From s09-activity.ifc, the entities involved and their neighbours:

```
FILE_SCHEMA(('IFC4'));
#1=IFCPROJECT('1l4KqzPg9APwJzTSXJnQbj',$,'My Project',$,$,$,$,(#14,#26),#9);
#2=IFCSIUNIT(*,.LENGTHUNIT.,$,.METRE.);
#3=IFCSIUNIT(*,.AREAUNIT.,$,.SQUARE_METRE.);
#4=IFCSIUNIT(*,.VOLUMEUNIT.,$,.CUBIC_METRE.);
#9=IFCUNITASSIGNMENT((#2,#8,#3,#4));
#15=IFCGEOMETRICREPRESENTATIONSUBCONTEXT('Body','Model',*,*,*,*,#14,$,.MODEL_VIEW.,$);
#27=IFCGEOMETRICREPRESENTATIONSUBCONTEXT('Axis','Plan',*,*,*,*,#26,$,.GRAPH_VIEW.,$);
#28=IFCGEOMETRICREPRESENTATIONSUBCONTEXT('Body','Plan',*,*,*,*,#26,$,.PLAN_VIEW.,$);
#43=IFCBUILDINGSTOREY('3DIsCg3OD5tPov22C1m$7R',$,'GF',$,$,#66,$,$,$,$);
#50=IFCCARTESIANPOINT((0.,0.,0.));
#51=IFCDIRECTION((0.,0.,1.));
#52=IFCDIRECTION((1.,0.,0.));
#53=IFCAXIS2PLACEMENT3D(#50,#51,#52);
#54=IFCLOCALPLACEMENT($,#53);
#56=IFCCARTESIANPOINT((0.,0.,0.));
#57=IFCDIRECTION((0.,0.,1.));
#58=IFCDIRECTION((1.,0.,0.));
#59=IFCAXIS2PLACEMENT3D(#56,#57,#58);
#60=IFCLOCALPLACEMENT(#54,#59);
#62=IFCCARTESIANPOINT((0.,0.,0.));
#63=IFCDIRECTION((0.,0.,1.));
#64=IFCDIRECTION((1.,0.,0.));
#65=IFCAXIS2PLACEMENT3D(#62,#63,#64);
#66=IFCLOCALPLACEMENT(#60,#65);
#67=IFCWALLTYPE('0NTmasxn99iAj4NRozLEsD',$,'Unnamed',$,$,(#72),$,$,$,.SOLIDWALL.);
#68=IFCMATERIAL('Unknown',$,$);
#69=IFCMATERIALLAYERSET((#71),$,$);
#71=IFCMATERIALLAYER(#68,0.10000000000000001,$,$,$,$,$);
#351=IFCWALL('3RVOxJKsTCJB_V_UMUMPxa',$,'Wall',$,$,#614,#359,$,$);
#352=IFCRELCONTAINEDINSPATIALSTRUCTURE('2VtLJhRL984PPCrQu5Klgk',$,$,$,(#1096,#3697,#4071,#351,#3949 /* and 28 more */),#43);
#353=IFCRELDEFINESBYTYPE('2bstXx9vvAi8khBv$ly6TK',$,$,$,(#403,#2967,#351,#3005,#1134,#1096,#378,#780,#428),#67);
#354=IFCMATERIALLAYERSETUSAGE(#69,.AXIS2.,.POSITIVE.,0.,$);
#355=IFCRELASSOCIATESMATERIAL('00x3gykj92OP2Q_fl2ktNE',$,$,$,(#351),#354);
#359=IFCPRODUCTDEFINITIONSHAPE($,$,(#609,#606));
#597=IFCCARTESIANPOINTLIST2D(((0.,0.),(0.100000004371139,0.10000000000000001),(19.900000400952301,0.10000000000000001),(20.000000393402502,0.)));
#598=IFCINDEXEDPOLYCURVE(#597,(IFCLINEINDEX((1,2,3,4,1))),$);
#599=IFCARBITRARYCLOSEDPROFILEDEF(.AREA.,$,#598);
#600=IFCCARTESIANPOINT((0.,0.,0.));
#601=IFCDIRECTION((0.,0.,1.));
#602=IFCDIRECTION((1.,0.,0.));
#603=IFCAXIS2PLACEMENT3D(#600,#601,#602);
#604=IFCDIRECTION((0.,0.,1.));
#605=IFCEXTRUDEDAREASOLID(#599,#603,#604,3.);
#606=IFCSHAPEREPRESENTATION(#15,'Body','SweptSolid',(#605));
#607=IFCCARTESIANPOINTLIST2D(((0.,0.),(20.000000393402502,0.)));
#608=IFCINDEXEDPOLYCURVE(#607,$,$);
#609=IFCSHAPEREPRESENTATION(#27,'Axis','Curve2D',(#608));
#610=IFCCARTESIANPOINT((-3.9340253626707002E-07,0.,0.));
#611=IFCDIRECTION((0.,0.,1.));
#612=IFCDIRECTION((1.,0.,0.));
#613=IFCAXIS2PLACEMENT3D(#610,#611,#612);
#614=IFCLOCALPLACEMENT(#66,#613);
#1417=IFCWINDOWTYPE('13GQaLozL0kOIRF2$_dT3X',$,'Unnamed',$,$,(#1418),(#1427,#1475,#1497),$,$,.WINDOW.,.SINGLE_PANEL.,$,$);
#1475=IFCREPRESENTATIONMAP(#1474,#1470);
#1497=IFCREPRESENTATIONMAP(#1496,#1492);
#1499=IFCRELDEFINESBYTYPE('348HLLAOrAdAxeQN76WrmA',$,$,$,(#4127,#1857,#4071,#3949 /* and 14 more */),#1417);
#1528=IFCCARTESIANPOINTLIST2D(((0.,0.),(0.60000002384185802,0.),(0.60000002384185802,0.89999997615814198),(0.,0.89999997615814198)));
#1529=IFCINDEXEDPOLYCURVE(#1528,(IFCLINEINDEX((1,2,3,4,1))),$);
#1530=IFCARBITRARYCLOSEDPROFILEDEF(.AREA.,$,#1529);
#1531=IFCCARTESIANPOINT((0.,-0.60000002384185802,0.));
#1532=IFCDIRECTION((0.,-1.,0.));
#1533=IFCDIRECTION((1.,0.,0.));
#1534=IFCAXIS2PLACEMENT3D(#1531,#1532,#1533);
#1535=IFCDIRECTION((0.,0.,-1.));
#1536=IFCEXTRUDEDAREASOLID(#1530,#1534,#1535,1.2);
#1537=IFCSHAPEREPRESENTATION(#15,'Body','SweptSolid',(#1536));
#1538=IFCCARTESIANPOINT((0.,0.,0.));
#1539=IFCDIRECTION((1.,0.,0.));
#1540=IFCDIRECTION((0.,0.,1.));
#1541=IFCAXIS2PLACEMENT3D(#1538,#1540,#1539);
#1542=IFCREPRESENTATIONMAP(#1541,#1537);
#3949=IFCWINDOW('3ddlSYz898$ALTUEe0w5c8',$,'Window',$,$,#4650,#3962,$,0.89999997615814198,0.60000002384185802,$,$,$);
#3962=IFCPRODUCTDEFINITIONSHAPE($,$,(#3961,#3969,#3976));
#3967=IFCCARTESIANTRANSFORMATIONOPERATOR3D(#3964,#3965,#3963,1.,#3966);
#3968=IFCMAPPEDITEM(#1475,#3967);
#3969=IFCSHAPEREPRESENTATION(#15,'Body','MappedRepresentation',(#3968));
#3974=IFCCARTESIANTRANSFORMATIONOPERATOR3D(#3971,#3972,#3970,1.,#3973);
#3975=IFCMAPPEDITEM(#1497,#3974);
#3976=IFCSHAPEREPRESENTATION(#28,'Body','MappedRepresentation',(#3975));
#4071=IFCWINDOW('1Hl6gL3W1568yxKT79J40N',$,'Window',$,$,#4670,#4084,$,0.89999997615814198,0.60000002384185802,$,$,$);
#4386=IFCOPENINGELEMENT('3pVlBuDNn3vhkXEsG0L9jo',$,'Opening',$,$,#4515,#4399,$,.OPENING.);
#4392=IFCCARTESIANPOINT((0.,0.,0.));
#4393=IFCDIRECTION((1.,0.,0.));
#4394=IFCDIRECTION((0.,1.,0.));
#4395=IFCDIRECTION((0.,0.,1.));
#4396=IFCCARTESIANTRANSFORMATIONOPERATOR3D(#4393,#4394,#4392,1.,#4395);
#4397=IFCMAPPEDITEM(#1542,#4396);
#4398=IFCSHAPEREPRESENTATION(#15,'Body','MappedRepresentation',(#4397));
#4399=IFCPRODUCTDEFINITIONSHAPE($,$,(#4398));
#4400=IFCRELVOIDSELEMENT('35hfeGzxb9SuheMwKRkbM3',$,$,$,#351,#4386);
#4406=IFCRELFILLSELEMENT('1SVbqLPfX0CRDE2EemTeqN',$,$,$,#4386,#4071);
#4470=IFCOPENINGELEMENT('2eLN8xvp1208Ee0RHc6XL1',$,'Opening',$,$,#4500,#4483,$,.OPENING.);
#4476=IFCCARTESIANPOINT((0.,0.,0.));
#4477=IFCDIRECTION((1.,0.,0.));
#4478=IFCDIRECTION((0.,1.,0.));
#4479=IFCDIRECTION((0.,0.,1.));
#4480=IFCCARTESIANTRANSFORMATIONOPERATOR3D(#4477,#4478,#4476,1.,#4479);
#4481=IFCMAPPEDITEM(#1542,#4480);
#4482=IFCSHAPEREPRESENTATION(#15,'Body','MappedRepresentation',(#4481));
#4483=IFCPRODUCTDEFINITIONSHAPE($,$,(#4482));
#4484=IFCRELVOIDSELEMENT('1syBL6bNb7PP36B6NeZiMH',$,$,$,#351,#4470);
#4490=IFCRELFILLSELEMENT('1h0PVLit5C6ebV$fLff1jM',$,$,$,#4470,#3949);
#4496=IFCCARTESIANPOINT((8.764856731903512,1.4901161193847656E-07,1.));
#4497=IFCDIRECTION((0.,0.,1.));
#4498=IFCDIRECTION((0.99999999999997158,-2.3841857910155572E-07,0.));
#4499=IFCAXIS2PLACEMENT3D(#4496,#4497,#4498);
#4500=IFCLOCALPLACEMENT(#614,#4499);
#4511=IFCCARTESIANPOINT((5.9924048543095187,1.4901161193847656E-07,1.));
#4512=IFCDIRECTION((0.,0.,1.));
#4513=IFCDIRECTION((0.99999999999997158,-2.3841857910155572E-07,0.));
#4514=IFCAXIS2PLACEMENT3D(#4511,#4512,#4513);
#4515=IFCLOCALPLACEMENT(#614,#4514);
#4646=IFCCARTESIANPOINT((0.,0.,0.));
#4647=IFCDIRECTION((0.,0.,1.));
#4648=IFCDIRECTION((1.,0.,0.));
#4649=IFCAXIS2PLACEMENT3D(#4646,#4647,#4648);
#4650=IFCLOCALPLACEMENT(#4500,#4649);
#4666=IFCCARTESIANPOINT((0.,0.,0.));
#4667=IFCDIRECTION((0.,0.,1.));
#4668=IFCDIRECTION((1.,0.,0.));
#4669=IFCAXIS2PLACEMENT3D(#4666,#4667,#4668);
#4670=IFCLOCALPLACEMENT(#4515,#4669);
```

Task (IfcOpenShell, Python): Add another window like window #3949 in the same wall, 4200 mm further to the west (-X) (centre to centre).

```python
import ifcopenshell
import ifcopenshell.api.feature
import ifcopenshell.api.geometry
import ifcopenshell.api.root
import ifcopenshell.geom
import ifcopenshell.util.element
import ifcopenshell.util.placement
import ifcopenshell.util.shape
import ifcopenshell.util.unit

model = ifcopenshell.open("s09-activity.ifc")
unit_scale = ifcopenshell.util.unit.calculate_unit_scale(model)
settings = ifcopenshell.geom.settings()


def volume(element):
    """Net volume in cubic metres, openings subtracted."""
    shape = ifcopenshell.geom.create_shape(settings, element)
    return ifcopenshell.util.shape.get_volume(shape.geometry)


window = model.by_id(3949)
opening = window.FillsVoids[0].RelatingOpeningElement
wall = opening.VoidsElements[0].RelatingBuildingElement
before = volume(wall)
shift = ifcopenshell.util.placement.get_local_placement(wall.ObjectPlacement)[:3, 0] * -4.2 / unit_scale

# copy_class copies the void relationship, type, container and properties, but no geometry.
new_opening = ifcopenshell.api.root.copy_class(model, product=opening)
new_opening.Representation = ifcopenshell.util.element.copy_deep(
    model, opening.Representation, exclude=["IfcGeometricRepresentationContext", "IfcRepresentationMap"]
)
new_window = ifcopenshell.api.root.copy_class(model, product=window)
new_window.Representation = ifcopenshell.util.element.copy_deep(
    model, window.Representation, exclude=["IfcGeometricRepresentationContext", "IfcRepresentationMap"]
)
ifcopenshell.api.feature.add_filling(model, opening=new_opening, element=new_window)

for old, new in ((opening, new_opening), (window, new_window)):
    matrix = ifcopenshell.util.placement.get_local_placement(old.ObjectPlacement)
    matrix[:3, 3] += shift
    ifcopenshell.api.geometry.edit_object_placement(model, product=new, matrix=matrix, is_si=False)

after = volume(wall)

print(f"wall volume {before:.3f} -> {after:.3f} m3")

model.write("s09-activity_rev.ifc")
```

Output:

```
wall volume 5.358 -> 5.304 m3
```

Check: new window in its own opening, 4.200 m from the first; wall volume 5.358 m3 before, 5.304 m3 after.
